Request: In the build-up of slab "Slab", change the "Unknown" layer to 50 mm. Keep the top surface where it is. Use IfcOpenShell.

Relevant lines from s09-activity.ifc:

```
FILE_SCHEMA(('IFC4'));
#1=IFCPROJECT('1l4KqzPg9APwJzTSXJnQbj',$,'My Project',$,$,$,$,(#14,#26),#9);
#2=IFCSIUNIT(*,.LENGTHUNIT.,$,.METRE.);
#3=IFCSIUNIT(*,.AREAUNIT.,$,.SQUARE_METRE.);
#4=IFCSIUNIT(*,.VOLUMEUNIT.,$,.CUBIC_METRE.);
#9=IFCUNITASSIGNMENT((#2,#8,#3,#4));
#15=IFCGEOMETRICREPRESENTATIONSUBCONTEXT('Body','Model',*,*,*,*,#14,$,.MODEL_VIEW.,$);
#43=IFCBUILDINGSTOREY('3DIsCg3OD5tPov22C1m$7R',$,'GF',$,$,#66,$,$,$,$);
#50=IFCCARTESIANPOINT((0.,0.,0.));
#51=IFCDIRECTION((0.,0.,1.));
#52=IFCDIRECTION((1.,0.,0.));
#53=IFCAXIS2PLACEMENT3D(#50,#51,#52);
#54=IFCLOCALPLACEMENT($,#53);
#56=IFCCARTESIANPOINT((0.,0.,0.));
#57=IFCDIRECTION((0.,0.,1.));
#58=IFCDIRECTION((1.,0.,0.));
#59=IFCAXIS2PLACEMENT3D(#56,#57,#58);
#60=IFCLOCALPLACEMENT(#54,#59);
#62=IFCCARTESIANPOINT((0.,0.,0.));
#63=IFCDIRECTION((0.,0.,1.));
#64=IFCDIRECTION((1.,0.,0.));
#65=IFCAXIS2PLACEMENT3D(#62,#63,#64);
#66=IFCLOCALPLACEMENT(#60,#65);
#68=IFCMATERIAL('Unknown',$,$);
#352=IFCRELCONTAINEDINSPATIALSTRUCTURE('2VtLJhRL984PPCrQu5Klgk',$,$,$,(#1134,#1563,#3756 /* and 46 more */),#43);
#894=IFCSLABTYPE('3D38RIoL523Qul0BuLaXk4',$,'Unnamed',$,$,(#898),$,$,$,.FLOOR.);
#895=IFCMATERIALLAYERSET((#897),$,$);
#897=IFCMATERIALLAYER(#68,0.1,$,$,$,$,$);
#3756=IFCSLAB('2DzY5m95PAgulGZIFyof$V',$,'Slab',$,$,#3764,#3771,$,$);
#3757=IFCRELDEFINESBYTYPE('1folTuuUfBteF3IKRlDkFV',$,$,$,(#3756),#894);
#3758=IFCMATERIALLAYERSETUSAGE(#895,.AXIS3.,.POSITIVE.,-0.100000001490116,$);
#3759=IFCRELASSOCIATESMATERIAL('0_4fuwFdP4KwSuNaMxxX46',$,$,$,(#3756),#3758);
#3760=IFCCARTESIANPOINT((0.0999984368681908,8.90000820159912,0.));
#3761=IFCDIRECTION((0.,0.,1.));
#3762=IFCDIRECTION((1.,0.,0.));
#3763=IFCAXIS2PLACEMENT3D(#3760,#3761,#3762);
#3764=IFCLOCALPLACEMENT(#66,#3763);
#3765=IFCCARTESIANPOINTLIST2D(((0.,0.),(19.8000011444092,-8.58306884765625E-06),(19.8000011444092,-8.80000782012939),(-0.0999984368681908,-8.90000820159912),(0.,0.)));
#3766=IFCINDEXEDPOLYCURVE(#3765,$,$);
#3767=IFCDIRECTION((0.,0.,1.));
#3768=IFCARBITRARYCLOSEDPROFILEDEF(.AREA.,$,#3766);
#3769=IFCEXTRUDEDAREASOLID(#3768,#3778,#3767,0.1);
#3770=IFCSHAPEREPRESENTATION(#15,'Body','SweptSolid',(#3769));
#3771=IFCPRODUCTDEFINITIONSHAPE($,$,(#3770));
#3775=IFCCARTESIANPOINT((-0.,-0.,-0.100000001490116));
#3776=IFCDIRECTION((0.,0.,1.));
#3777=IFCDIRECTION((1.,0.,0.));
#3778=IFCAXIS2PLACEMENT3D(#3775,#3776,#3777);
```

```python
import ifcopenshell
import ifcopenshell.util.element
import ifcopenshell.util.representation
import ifcopenshell.util.unit

model = ifcopenshell.open("s09-activity.ifc")
unit_scale = ifcopenshell.util.unit.calculate_unit_scale(model)

layer_set = model.by_id(895)
layer = next(l for l in layer_set.MaterialLayers if l.Material and l.Material.Name == "Unknown")
change = 0.05 / unit_scale - layer.LayerThickness
layer.LayerThickness += change

# Geometry does not follow the layer set by itself.
slabs = [e for e in ifcopenshell.util.element.get_elements_by_material(model, layer_set) if e.is_a("IfcSlab")]
for slab in sorted(slabs, key=lambda e: e.id()):
    body = ifcopenshell.util.representation.get_representation(slab, "Model", "Body")
    solid = body.Items[0]
    old_depth = solid.Depth
    solid.Depth += change
    # Extruded upwards: lower the start of the extrusion so the top stays.
    x, y, z = solid.Position.Location.Coordinates
    solid.Position.Location = model.createIfcCartesianPoint((x, y, z - change))
    print(slab.id(), f"{old_depth:g} -> {solid.Depth:g}")

# The layers are counted up from the underside, which has moved.
for usage in {ifcopenshell.util.element.get_material(slab) for slab in slabs}:
    usage.OffsetFromReferenceLine -= change

model.write("s09-activity_updated.ifc")
```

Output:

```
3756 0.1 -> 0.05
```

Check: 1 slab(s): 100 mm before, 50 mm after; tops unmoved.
